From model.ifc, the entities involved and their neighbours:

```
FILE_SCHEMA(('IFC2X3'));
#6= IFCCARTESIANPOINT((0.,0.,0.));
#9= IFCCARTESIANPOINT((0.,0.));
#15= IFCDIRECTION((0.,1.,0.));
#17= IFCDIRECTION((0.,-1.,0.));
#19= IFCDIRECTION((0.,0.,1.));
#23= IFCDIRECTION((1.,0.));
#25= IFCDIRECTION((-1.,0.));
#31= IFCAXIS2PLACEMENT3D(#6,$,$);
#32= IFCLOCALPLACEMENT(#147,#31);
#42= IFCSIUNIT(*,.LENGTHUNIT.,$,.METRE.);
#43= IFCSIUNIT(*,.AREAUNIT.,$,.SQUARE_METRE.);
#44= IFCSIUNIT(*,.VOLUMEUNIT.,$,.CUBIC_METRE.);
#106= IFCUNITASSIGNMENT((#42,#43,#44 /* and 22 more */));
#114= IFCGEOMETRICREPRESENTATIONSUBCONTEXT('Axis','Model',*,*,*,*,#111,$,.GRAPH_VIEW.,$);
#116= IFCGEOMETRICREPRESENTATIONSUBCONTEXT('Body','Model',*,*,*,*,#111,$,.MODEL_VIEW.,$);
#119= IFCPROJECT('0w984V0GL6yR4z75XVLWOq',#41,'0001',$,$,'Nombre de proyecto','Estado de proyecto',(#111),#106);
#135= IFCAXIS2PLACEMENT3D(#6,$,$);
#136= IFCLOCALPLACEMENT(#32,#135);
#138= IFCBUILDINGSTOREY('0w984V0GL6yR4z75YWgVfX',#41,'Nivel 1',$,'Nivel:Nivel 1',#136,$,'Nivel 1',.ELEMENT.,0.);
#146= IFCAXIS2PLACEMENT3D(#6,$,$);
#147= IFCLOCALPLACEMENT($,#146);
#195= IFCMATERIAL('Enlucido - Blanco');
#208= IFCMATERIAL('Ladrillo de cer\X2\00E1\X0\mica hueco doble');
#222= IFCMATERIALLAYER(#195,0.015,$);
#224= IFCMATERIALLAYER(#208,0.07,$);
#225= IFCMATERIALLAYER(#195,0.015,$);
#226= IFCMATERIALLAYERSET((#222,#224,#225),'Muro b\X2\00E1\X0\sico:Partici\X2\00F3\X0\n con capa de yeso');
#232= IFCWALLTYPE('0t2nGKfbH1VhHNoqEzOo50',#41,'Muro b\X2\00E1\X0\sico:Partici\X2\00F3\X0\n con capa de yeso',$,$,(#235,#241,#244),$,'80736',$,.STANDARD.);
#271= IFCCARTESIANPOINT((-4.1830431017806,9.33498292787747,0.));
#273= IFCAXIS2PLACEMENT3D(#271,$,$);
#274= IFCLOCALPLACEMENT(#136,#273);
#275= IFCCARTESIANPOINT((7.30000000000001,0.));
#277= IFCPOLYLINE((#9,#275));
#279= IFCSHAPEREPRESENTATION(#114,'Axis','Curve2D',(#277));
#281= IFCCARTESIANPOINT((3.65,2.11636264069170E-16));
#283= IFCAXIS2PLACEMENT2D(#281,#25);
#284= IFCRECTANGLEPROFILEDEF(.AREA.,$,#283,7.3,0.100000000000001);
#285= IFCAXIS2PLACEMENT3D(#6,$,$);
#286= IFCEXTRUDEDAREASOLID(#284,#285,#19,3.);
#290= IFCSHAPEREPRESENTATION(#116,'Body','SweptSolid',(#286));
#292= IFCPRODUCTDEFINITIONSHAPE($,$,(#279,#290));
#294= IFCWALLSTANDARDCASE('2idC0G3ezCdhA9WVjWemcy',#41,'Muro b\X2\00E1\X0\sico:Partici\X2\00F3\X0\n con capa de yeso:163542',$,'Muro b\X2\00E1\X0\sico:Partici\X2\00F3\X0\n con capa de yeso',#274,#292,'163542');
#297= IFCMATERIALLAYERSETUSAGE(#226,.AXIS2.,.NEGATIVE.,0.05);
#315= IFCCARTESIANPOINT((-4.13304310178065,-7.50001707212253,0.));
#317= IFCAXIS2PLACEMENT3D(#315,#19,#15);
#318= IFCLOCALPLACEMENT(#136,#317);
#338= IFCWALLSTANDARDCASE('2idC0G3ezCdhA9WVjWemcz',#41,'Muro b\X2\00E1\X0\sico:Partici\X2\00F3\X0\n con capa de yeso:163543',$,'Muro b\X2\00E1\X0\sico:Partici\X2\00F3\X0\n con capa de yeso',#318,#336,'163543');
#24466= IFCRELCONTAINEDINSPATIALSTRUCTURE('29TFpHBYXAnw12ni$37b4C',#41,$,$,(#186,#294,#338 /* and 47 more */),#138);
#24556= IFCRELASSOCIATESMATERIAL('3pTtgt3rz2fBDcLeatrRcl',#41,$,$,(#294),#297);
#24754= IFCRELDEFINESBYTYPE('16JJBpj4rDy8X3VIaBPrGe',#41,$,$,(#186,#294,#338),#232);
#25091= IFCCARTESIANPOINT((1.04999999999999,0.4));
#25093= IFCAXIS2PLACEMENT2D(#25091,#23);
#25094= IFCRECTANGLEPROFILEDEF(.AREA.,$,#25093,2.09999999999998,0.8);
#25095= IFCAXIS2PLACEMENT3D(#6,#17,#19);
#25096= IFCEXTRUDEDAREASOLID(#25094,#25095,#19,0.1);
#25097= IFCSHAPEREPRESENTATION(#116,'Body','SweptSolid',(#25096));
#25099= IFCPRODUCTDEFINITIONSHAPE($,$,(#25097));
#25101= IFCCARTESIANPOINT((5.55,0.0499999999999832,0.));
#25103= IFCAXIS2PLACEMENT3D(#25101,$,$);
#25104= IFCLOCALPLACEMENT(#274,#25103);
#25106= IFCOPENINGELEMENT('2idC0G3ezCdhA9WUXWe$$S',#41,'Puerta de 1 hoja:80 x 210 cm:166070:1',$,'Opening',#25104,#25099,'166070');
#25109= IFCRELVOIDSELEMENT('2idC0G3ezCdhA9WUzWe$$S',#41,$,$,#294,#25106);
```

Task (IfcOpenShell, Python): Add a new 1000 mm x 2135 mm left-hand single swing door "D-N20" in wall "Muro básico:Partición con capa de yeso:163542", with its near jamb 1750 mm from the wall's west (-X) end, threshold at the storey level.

```python
import numpy as np
import ifcopenshell
import ifcopenshell.api.feature
import ifcopenshell.api.geometry
import ifcopenshell.api.root
import ifcopenshell.api.spatial
import ifcopenshell.api.type
import ifcopenshell.geom
import ifcopenshell.util.element
import ifcopenshell.util.placement
import ifcopenshell.util.representation
import ifcopenshell.util.shape
import ifcopenshell.util.unit

model = ifcopenshell.open("model.ifc")
unit_scale = ifcopenshell.util.unit.calculate_unit_scale(model)
settings = ifcopenshell.geom.settings()


def volume(element):
    """Net volume in cubic metres, openings subtracted."""
    shape = ifcopenshell.geom.create_shape(settings, element)
    return ifcopenshell.util.shape.get_volume(shape.geometry)


wall = model.by_id(294)
storey = ifcopenshell.util.element.get_container(wall, ifc_class="IfcBuildingStorey")
context = ifcopenshell.util.representation.get_context(model, "Model", "Body", "MODEL_VIEW")
before = volume(wall)

width, height, from_end, sill = 1, 2.135, 1.75, 0.0  # metres

# The wall runs along its own X axis, and the end named is its -X end.
wall_shape = ifcopenshell.geom.create_shape(settings, wall)
x, y, z = ifcopenshell.util.shape.get_vertices(wall_shape.geometry).T
start = x.min() + from_end
face, thickness = float(y.min()), float(y.max() - y.min())
wall_matrix = ifcopenshell.util.placement.get_local_placement(wall.ObjectPlacement)
level = ifcopenshell.util.placement.get_local_placement(storey.ObjectPlacement)[2, 3]


def in_wall(x, y):
    """Placement at x, y metres in the wall's axes, at sill height."""
    matrix = wall_matrix.copy()
    matrix[:, 3] = wall_matrix @ np.array([x / unit_scale, y / unit_scale, 0.0, 1.0])
    matrix[2, 3] = level + sill / unit_scale
    return matrix


# Opening: a box that overshoots both wall faces by 50 mm.
opening = ifcopenshell.api.root.create_entity(model, ifc_class="IfcOpeningElement")
box = ifcopenshell.api.geometry.add_wall_representation(
    model, context=context, length=width, height=height, thickness=thickness + 0.1
)
ifcopenshell.api.geometry.assign_representation(model, product=opening, representation=box)
ifcopenshell.api.geometry.edit_object_placement(model, product=opening, matrix=in_wall(start, face - 0.05), is_si=False)
ifcopenshell.api.feature.add_feature(model, feature=opening, element=wall)

door = ifcopenshell.api.root.create_entity(model, ifc_class="IfcDoor", name="D-N20")
door.OverallWidth, door.OverallHeight = width / unit_scale, height / unit_scale
body = ifcopenshell.api.geometry.add_door_representation(
    model,
    context=context,
    overall_width=door.OverallWidth,
    overall_height=door.OverallHeight,
    operation_type="SINGLE_SWING_LEFT",
    lining_properties={"LiningDepth": thickness / unit_scale, "ThresholdDepth": thickness / unit_scale},
)
ifcopenshell.api.geometry.assign_representation(model, product=door, representation=body)
ifcopenshell.api.spatial.assign_container(model, products=[door], relating_structure=storey)
fills = ifcopenshell.api.feature.add_filling(model, opening=opening, element=door)
fills.OwnerHistory = door.OwnerHistory  # required in IFC2X3

# IFC2X3 keeps the operation on the door style.
style = ifcopenshell.api.root.create_entity(model, ifc_class="IfcDoorStyle", name="D-N20")
style.OperationType, style.ConstructionType = "SINGLE_SWING_LEFT", "NOTDEFINED"
style.ParameterTakesPrecedence = style.Sizeable = False
ifcopenshell.api.type.assign_type(model, related_objects=[door], relating_type=style)

# The lining spans the wall, so the door starts at the wall face.
ifcopenshell.api.geometry.edit_object_placement(model, product=door, matrix=in_wall(start, face), is_si=False)

after = volume(wall)

print(f"wall volume {before:.3f} -> {after:.3f} m3")

model.write("model_updated.ifc")
```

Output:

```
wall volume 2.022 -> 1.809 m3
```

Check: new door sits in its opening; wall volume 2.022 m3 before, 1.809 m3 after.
